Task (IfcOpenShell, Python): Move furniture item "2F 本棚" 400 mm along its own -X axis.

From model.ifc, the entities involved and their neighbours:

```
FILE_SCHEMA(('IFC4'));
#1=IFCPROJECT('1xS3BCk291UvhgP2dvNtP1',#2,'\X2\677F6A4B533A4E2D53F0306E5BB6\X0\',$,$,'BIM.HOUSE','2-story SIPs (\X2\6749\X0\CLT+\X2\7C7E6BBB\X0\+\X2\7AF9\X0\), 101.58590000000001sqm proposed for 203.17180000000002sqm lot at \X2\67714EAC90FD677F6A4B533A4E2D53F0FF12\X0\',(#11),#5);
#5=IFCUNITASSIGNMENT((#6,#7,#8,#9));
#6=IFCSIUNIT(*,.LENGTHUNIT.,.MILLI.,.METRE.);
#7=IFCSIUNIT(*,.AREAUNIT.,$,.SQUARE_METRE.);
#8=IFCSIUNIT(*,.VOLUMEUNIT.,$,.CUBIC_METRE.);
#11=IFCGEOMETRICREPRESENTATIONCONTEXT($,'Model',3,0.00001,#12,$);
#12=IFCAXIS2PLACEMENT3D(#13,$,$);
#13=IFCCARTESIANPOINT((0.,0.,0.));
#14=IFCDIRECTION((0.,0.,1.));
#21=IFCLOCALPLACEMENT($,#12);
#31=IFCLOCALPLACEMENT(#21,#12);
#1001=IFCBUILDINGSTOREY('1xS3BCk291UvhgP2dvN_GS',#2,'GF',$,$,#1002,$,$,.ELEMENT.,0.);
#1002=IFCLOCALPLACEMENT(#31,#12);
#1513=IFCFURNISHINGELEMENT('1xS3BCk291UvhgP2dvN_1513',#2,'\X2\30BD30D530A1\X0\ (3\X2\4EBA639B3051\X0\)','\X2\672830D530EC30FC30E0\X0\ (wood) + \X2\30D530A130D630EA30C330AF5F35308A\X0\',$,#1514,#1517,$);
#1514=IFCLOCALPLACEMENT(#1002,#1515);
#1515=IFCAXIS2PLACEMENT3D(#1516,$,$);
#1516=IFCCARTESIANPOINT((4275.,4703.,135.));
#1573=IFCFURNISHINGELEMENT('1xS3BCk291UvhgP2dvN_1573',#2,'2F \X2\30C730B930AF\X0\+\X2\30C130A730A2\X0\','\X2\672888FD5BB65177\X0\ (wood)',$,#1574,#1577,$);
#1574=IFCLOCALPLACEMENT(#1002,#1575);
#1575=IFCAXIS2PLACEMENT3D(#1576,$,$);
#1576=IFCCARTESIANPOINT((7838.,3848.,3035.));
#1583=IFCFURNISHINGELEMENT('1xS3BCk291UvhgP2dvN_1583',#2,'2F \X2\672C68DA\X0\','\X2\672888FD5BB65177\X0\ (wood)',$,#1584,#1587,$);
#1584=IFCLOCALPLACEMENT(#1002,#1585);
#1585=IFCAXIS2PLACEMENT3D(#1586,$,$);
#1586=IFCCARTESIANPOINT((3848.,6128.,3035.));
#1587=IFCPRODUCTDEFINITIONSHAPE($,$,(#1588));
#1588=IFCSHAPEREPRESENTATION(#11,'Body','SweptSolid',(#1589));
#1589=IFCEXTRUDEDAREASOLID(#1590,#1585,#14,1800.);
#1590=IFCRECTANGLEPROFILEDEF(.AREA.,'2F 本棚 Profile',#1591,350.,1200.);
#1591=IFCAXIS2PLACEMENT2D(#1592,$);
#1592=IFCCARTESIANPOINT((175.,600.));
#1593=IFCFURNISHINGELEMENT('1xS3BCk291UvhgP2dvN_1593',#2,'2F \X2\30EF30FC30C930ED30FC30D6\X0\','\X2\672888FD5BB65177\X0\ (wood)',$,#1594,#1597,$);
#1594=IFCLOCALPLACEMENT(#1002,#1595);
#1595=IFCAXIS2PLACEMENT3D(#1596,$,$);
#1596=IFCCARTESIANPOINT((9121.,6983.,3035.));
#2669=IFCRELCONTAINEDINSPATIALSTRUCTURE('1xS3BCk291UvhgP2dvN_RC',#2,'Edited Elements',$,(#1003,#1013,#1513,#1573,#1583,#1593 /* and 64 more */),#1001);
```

```python
import ifcopenshell
import ifcopenshell.api.geometry
import ifcopenshell.util.placement

model = ifcopenshell.open("model.ifc")

item = model.by_guid("1xS3BCk291UvhgP2dvN_1583")
matrix = ifcopenshell.util.placement.get_local_placement(item.ObjectPlacement)
matrix[:3, 3] -= matrix[:3, 0] * 400.0
ifcopenshell.api.geometry.edit_object_placement(model, product=item, matrix=matrix, is_si=False)

print(ifcopenshell.util.placement.get_local_placement(item.ObjectPlacement).round(3) + 0.0)

model.write("model_rev.ifc")
```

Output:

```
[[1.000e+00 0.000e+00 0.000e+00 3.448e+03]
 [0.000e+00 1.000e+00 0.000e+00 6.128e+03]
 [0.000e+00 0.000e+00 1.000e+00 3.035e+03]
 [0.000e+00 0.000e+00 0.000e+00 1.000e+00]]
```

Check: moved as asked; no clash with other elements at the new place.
